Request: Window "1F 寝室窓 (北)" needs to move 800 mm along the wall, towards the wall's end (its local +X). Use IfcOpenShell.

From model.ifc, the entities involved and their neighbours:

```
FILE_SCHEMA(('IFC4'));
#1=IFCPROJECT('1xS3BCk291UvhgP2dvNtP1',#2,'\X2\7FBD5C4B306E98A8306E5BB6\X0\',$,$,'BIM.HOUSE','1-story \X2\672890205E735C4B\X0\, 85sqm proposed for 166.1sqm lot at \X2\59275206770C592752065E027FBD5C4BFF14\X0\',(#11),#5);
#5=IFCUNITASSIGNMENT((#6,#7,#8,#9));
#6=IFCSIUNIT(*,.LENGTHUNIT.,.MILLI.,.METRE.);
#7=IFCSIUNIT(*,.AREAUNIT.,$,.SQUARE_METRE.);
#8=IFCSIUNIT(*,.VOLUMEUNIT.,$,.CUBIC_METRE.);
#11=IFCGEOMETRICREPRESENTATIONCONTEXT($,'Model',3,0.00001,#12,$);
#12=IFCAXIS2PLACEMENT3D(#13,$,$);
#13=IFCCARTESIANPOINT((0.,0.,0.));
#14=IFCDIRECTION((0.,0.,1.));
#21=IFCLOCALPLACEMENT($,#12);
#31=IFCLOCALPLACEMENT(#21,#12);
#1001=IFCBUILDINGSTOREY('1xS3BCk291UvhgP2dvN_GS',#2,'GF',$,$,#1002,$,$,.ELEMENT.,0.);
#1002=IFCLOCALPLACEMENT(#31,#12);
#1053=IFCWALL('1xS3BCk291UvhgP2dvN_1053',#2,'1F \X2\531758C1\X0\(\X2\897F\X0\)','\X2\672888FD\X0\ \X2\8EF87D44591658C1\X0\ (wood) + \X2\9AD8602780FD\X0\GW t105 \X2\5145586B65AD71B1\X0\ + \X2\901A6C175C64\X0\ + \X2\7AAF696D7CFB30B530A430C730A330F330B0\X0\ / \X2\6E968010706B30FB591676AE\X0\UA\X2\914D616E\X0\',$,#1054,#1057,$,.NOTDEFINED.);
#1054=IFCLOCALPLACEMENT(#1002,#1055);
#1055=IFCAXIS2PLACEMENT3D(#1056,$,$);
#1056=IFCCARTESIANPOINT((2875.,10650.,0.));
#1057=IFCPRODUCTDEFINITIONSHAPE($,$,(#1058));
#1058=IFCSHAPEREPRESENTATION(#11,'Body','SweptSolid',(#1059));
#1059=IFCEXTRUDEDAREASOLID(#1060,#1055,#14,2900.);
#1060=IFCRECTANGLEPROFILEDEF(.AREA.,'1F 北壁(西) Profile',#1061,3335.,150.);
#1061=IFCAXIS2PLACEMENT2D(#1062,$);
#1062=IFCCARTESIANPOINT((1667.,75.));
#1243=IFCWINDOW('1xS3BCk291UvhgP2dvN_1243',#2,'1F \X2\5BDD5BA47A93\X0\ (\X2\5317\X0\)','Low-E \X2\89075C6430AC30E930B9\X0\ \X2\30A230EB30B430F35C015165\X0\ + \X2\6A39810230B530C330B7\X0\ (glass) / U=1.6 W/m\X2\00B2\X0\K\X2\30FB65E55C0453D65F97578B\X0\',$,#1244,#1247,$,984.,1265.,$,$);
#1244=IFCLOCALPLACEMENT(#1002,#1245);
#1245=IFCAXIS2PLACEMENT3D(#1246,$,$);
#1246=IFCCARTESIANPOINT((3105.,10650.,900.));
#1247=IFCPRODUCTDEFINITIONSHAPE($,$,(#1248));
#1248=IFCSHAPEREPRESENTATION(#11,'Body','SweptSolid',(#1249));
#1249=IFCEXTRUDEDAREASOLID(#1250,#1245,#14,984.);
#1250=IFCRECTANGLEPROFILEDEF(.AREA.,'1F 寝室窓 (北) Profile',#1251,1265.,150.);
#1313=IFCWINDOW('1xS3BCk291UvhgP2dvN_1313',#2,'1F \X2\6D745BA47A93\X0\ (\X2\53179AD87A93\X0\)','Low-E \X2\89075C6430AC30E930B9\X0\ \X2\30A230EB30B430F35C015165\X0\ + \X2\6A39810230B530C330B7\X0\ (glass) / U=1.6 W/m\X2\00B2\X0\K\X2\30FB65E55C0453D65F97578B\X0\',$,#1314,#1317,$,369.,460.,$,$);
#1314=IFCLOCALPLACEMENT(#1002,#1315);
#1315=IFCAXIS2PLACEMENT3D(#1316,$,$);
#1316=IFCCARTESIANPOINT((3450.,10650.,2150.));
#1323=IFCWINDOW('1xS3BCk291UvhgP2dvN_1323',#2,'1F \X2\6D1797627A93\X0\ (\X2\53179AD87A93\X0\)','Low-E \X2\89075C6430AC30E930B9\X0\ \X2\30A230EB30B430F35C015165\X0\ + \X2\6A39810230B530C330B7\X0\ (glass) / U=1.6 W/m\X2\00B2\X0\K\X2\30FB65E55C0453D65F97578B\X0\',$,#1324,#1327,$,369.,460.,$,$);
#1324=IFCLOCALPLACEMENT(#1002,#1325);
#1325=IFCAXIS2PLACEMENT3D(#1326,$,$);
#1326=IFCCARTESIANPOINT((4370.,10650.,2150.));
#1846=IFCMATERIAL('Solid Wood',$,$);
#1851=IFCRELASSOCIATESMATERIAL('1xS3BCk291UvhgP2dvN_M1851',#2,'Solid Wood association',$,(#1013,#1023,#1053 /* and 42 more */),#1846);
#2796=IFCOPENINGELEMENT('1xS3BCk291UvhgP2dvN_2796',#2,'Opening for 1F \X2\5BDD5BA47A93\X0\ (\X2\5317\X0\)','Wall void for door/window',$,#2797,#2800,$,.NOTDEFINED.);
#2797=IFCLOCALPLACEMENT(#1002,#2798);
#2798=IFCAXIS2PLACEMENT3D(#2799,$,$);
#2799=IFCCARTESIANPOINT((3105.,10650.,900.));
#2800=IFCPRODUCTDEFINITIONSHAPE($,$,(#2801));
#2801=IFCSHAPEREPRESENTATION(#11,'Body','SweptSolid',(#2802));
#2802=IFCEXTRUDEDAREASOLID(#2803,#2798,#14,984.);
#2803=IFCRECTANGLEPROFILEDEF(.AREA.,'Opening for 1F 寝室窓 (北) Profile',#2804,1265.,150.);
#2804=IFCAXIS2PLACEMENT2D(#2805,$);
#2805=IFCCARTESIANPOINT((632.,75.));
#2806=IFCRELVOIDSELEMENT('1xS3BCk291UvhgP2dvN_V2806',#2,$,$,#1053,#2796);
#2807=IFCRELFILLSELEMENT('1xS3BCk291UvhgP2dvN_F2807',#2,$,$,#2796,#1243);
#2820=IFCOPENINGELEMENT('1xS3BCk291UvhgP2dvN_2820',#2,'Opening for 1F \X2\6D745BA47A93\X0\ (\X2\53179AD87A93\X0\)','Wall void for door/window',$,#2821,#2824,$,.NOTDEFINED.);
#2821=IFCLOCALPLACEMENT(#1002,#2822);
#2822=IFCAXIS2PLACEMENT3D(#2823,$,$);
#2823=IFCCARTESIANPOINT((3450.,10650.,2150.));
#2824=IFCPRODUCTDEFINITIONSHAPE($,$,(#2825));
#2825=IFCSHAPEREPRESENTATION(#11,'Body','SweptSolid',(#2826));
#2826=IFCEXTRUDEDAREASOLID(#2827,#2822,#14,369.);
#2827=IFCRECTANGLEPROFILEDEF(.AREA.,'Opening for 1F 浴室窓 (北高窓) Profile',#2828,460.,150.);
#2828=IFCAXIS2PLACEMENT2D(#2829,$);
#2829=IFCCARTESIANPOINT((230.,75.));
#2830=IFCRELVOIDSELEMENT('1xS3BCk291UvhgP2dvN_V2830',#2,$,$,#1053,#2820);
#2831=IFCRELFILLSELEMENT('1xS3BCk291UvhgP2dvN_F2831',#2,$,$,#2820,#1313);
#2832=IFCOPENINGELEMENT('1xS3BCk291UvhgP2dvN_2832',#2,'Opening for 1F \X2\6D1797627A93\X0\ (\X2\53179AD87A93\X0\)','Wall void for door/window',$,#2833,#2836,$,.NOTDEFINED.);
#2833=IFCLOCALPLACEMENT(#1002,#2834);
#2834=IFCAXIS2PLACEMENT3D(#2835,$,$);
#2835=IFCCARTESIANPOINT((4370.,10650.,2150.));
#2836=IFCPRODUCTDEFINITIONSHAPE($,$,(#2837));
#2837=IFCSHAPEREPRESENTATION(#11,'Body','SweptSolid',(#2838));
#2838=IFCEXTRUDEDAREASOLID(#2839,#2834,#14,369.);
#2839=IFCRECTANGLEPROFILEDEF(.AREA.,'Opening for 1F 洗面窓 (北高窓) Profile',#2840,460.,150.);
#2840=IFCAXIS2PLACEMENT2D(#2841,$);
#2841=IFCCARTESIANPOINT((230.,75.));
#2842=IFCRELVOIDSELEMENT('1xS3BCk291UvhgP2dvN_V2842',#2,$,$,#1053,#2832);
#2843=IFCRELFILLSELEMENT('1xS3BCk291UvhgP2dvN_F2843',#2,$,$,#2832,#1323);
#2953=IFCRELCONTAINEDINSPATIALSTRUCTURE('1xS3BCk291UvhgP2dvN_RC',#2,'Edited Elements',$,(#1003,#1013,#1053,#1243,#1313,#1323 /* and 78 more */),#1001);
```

```python
import ifcopenshell
import ifcopenshell.api.geometry
import ifcopenshell.util.placement

model = ifcopenshell.open("model.ifc")

window = model.by_guid("1xS3BCk291UvhgP2dvN_1243")
opening = window.FillsVoids[0].RelatingOpeningElement
wall = opening.VoidsElements[0].RelatingBuildingElement

wall_matrix = ifcopenshell.util.placement.get_local_placement(wall.ObjectPlacement)
shift = wall_matrix[:3, 0] * 800.0
before = ifcopenshell.util.placement.get_local_placement(window.ObjectPlacement)[:3, 3].copy()

# The window is not placed relative to its opening, so move both.
for product in (opening, window):
    matrix = ifcopenshell.util.placement.get_local_placement(product.ObjectPlacement)
    matrix[:3, 3] += shift
    ifcopenshell.api.geometry.edit_object_placement(model, product=product, matrix=matrix, is_si=False)

after = ifcopenshell.util.placement.get_local_placement(window.ObjectPlacement)[:3, 3]
print("window moved by", (after - before).round(3) + 0.0)

model.write("model_rev.ifc")
```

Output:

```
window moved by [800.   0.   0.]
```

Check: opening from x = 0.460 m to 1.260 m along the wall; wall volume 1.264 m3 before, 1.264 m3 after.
